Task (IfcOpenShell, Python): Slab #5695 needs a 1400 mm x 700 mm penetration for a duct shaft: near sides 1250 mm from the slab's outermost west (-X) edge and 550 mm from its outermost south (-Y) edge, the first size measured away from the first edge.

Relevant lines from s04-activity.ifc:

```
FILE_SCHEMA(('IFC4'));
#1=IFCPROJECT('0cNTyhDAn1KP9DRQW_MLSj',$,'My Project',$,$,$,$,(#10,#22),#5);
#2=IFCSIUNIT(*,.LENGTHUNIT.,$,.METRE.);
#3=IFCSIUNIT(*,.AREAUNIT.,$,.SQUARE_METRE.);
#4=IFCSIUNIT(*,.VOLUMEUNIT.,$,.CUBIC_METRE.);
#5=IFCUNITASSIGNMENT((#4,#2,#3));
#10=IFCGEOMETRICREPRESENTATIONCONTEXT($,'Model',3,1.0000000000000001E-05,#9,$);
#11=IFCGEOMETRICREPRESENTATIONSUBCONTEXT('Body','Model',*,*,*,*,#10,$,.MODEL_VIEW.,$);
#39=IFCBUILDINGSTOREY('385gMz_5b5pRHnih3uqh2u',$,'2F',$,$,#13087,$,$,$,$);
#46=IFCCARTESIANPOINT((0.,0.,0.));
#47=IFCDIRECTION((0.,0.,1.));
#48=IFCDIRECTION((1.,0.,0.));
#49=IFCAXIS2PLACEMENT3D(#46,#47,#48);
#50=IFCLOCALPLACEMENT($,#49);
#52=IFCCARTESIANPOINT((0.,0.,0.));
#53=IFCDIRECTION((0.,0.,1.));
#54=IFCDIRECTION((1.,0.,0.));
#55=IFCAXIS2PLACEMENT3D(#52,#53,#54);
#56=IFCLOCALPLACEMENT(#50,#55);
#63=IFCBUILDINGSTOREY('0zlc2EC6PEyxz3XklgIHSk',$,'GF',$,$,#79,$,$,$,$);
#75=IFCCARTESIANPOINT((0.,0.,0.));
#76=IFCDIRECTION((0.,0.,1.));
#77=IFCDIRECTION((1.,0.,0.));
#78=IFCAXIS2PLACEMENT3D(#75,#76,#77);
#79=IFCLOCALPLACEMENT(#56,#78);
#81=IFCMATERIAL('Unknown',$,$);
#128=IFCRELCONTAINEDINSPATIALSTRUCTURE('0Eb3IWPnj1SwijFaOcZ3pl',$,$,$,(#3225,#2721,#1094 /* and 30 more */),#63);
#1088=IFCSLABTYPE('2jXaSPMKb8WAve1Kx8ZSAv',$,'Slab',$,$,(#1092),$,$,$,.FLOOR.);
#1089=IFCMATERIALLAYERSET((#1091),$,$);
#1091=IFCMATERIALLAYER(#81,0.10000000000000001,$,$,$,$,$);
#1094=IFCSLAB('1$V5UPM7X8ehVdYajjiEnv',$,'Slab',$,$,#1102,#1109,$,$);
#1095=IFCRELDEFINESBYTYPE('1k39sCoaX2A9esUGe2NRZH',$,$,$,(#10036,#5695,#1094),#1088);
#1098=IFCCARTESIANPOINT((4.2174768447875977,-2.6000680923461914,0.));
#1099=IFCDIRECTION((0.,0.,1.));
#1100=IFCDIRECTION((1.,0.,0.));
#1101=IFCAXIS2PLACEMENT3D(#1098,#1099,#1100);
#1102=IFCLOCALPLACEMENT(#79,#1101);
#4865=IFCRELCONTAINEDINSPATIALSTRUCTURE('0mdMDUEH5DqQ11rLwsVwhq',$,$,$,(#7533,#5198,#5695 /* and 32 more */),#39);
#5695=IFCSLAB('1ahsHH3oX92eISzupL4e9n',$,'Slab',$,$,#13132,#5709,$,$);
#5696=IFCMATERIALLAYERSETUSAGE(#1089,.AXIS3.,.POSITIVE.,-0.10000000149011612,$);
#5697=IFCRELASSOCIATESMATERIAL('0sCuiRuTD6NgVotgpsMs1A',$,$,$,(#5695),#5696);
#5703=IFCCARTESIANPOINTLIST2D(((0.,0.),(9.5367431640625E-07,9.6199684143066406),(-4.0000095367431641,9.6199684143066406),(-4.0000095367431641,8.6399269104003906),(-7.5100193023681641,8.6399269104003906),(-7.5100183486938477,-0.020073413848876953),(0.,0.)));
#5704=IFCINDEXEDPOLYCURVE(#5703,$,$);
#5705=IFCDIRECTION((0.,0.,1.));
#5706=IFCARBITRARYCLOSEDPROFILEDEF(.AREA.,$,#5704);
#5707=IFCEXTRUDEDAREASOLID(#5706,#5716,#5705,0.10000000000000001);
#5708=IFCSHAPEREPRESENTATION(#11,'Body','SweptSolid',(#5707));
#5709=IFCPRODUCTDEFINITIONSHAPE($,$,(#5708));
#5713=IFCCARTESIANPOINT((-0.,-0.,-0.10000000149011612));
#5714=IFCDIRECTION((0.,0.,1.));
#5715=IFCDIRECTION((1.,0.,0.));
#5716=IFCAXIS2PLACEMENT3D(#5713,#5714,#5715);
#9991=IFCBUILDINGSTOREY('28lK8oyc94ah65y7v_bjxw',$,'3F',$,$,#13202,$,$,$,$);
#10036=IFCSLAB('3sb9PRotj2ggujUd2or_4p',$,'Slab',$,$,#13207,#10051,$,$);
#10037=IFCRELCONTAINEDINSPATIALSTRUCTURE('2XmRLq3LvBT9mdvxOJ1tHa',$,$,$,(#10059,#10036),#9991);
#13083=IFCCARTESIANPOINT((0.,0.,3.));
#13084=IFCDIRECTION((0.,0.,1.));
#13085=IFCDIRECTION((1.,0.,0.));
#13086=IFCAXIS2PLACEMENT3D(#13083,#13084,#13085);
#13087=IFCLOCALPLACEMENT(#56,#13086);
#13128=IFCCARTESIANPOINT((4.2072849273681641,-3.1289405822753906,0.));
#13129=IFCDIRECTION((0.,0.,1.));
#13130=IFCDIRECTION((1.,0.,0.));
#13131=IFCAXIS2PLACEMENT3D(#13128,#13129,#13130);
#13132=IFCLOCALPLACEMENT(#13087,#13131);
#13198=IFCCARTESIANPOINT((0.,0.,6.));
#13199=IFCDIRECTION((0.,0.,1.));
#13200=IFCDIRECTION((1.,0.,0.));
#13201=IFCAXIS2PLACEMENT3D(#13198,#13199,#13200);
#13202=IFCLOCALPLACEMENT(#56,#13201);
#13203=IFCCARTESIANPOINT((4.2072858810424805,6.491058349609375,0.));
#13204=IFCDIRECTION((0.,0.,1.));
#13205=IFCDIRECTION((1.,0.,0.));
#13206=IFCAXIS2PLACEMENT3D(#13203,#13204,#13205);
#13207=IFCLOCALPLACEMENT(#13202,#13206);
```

```python
import numpy as np
import ifcopenshell
import ifcopenshell.api.feature
import ifcopenshell.api.geometry
import ifcopenshell.api.root
import ifcopenshell.geom
import ifcopenshell.util.placement
import ifcopenshell.util.representation
import ifcopenshell.util.shape
import ifcopenshell.util.unit

model = ifcopenshell.open("s04-activity.ifc")
unit_scale = ifcopenshell.util.unit.calculate_unit_scale(model)
settings = ifcopenshell.geom.settings()


def volume(element):
    """Net volume in cubic metres, openings subtracted."""
    shape = ifcopenshell.geom.create_shape(settings, element)
    return ifcopenshell.util.shape.get_volume(shape.geometry)


slab = model.by_guid("1ahsHH3oX92eISzupL4e9n")
before = volume(slab)

# Extent in the slab's own axes, in metres. The edges named are its -X and -Y sides.
slab_shape = ifcopenshell.geom.create_shape(settings, slab)
vertices = ifcopenshell.util.shape.get_vertices(slab_shape.geometry)
x_min, y_min, bottom = vertices.min(axis=0)
top = vertices[:, 2].max()

opening = ifcopenshell.api.root.create_entity(model, ifc_class="IfcOpeningElement", name="Duct shaft opening", predefined_type="OPENING")
context = ifcopenshell.util.representation.get_context(model, "Model", "Body", "MODEL_VIEW")
width, depth = 1.4, 0.7
outline = [(0.0, 0.0), (width, 0.0), (width, depth), (0.0, depth), (0.0, 0.0)]
# Overshoot both faces by 50 mm so the cut is clean.
shape = ifcopenshell.api.geometry.add_slab_representation(
    model, context=context, depth=top - bottom + 0.1, polyline=outline
)
ifcopenshell.api.geometry.assign_representation(model, product=opening, representation=shape)

matrix = ifcopenshell.util.placement.get_local_placement(slab.ObjectPlacement)
matrix[:, 3] = matrix @ np.append(np.array([x_min + 1.25, y_min + 0.55, bottom - 0.05]) / unit_scale, 1.0)
ifcopenshell.api.geometry.edit_object_placement(model, product=opening, matrix=matrix, is_si=False)
ifcopenshell.api.feature.add_feature(model, feature=opening, element=slab)

after = volume(slab)

print(f"slab volume {before:.3f} -> {after:.3f} m3")

model.write("s04-activity-out.ifc")
```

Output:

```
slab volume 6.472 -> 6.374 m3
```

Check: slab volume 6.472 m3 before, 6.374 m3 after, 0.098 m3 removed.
